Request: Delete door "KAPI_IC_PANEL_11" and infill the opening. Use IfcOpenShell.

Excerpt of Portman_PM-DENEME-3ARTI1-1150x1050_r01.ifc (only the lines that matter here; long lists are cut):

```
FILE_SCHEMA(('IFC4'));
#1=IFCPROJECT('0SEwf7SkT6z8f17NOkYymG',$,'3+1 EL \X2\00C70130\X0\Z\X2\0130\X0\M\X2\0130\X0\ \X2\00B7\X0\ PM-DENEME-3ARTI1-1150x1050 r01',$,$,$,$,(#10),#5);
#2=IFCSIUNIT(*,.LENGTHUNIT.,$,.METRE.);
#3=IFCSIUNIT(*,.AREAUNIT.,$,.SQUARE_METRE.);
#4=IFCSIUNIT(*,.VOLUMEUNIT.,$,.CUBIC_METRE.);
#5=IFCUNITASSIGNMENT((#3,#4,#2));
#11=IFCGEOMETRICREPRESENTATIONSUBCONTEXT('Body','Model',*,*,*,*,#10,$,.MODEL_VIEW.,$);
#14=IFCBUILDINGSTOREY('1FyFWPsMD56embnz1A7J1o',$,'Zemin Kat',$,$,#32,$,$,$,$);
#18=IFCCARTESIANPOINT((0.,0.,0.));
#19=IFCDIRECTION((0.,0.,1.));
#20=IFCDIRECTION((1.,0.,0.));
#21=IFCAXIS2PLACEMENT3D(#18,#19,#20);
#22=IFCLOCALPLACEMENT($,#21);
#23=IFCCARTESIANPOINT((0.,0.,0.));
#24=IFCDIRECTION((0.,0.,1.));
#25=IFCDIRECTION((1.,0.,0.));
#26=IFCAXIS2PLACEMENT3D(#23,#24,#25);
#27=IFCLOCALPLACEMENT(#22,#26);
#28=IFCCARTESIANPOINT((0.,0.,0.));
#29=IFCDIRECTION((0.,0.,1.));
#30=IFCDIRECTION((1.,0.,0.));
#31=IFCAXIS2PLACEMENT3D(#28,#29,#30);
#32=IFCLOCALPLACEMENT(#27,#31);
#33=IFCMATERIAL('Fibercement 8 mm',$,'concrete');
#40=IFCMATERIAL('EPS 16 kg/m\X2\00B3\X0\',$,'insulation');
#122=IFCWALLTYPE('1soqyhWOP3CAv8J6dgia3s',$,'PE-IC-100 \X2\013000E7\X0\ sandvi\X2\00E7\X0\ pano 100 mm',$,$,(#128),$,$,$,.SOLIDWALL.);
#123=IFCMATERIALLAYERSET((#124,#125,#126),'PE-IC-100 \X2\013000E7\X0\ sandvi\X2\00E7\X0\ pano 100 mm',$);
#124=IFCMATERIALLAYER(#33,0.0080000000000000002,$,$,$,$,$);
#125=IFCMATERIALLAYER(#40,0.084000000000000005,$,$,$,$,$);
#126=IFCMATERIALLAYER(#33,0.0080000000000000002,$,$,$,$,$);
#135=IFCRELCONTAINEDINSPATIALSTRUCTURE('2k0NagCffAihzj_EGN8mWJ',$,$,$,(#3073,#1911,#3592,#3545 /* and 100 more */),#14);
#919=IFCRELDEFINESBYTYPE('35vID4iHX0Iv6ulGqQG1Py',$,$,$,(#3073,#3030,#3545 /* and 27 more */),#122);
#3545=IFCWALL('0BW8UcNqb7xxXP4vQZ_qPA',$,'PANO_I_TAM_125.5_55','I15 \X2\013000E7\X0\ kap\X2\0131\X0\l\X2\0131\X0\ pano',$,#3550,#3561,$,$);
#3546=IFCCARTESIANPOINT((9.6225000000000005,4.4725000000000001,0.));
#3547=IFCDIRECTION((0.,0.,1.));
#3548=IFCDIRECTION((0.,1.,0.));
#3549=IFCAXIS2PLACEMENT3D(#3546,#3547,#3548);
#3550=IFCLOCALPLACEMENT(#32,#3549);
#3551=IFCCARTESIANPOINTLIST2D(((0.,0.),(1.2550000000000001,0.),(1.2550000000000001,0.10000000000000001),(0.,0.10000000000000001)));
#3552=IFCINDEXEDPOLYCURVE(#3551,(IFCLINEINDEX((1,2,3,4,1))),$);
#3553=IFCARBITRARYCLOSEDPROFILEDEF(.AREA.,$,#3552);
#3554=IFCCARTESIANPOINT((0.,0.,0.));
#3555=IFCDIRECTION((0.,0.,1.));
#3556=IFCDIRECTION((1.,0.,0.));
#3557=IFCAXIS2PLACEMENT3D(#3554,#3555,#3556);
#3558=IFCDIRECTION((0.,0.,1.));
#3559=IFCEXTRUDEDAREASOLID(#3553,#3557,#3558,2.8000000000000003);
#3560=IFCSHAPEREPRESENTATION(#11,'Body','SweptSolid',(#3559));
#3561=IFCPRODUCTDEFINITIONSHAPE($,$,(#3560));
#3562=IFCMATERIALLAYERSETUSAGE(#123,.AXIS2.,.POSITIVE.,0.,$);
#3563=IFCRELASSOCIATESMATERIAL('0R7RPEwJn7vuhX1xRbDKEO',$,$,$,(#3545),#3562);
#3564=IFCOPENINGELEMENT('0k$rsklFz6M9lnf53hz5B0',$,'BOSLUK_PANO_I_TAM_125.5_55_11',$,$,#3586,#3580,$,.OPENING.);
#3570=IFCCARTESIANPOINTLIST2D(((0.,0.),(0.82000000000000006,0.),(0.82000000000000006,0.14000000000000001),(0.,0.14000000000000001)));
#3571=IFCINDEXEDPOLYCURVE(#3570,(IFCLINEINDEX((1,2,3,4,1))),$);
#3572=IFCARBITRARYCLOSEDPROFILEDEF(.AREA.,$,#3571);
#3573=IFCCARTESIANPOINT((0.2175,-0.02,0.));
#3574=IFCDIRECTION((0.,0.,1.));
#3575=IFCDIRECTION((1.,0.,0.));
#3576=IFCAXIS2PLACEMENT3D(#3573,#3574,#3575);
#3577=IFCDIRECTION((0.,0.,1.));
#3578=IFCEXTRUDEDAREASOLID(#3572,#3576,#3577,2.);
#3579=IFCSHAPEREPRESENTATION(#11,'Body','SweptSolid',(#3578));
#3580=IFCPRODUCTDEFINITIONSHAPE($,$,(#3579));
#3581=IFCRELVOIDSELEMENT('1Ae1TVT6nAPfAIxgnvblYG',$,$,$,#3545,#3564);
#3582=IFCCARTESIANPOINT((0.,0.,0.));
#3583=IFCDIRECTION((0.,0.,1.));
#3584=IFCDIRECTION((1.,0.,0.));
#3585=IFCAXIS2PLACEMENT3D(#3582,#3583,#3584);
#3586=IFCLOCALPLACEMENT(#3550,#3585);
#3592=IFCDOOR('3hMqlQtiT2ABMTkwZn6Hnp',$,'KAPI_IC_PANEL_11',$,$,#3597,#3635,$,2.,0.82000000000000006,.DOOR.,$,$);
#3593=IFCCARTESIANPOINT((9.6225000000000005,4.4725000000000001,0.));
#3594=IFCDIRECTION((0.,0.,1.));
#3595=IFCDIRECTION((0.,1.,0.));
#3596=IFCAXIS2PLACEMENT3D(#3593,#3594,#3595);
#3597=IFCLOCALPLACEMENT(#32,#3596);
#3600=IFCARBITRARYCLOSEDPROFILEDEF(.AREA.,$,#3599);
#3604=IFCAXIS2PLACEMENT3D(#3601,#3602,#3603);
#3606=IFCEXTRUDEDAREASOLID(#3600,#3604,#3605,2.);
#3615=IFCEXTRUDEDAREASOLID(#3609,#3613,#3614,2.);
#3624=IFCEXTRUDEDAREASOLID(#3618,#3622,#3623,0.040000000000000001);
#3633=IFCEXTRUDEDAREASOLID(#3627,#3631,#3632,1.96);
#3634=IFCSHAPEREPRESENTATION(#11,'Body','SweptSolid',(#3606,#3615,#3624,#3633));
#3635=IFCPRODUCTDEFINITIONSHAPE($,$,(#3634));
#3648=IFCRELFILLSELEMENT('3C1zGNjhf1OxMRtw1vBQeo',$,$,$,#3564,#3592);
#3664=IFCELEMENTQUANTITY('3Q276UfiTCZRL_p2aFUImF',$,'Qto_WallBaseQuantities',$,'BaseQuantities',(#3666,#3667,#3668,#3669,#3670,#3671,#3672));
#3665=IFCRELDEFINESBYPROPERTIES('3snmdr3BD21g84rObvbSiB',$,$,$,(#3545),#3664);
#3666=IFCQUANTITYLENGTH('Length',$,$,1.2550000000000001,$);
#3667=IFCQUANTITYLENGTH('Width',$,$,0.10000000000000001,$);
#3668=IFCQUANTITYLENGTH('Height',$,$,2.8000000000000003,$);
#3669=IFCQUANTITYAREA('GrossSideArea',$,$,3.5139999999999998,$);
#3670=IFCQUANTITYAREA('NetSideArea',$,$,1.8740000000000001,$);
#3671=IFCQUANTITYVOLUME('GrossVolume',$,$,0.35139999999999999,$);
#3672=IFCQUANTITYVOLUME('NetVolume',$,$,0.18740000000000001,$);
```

```python
import ifcopenshell
import ifcopenshell.api.feature
import ifcopenshell.api.pset
import ifcopenshell.api.root
import ifcopenshell.geom
import ifcopenshell.util.element
import ifcopenshell.util.shape
import ifcopenshell.util.unit

model = ifcopenshell.open("Portman_PM-DENEME-3ARTI1-1150x1050_r01.ifc")
area_scale = ifcopenshell.util.unit.calculate_unit_scale(model, "AREAUNIT")
volume_scale = ifcopenshell.util.unit.calculate_unit_scale(model, "VOLUMEUNIT")
settings = ifcopenshell.geom.settings()


def volume(element):
    """Net volume in cubic metres, openings subtracted."""
    shape = ifcopenshell.geom.create_shape(settings, element)
    return ifcopenshell.util.shape.get_volume(shape.geometry)


door = model.by_id(3592)
opening = door.FillsVoids[0].RelatingOpeningElement
wall = opening.VoidsElements[0].RelatingBuildingElement
before = volume(wall)

ifcopenshell.api.root.remove_product(model, product=door)
ifcopenshell.api.feature.remove_feature(model, feature=opening)

after = volume(wall)
thickness = 0.1  # wall thickness in metres

# Update the wall's stored quantities.
qto = model.by_id(ifcopenshell.util.element.get_pset(wall, "Qto_WallBaseQuantities", should_inherit=False)["id"])
ifcopenshell.api.pset.edit_qto(model, qto=qto, properties={
    "NetSideArea": after / thickness / area_scale,
    "NetVolume": after / volume_scale,
})

print(f"wall volume {before:.3f} -> {after:.3f} m3")

model.write("Portman_PM-DENEME-3ARTI1-1150x1050_r01_edited.ifc")
```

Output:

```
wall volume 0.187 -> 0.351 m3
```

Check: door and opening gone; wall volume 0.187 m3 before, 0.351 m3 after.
